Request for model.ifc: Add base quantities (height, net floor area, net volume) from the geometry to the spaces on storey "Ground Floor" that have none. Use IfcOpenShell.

First a look at what the model holds.

```python
import ifcopenshell
import ifcopenshell.util.element
import ifcopenshell.util.unit

model = ifcopenshell.open("model.ifc")
print(model.schema)
for unit_type in ("LENGTHUNIT", "AREAUNIT", "VOLUMEUNIT"):
    print(unit_type, ifcopenshell.util.unit.calculate_unit_scale(model, unit_type))
storey = next(s for s in model.by_type("IfcBuildingStorey") if s.Name == "Ground Floor")
spaces = [e for e in ifcopenshell.util.element.get_decomposition(storey) if e.is_a("IfcSpace")]
for e in sorted(spaces, key=lambda e: e.id()):
    print(e.id(), e.is_a(), e.Name, list(ifcopenshell.util.element.get_psets(e, qtos_only=True)), sep=" | ")
```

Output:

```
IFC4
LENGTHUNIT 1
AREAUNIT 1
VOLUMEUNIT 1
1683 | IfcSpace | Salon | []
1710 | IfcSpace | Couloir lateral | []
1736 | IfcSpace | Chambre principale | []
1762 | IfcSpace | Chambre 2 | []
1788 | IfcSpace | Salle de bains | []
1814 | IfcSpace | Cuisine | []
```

```python
import ifcopenshell
import ifcopenshell.api.pset
import ifcopenshell.geom
import ifcopenshell.util.element
import ifcopenshell.util.shape
import ifcopenshell.util.unit

model = ifcopenshell.open("model.ifc")
unit_scale = ifcopenshell.util.unit.calculate_unit_scale(model)
area_scale = ifcopenshell.util.unit.calculate_unit_scale(model, "AREAUNIT")
volume_scale = ifcopenshell.util.unit.calculate_unit_scale(model, "VOLUMEUNIT")
settings = ifcopenshell.geom.settings()

storey = next(s for s in model.by_type("IfcBuildingStorey") if s.Name == "Ground Floor")
spaces = [e for e in ifcopenshell.util.element.get_decomposition(storey) if e.is_a("IfcSpace")]

for e in sorted(spaces, key=lambda e: e.id()):
    if ifcopenshell.util.element.get_psets(e, qtos_only=True, should_inherit=False):
        continue
    # Geometry comes back in metres, in the element's own axes.
    shape = ifcopenshell.geom.create_shape(settings, e)
    values = {
        "Height": ifcopenshell.util.shape.get_z(shape.geometry) / unit_scale,
        "NetFloorArea": ifcopenshell.util.shape.get_footprint_area(shape.geometry) / area_scale,
        "NetVolume": ifcopenshell.util.shape.get_volume(shape.geometry) / volume_scale,
    }
    qto = ifcopenshell.api.pset.add_qto(model, product=e, name="Qto_SpaceBaseQuantities")
    ifcopenshell.api.pset.edit_qto(model, qto=qto, properties=values)
    print(e.id(), {k: round(v, 3) for k, v in values.items()})

model.write("model_v2.ifc")
```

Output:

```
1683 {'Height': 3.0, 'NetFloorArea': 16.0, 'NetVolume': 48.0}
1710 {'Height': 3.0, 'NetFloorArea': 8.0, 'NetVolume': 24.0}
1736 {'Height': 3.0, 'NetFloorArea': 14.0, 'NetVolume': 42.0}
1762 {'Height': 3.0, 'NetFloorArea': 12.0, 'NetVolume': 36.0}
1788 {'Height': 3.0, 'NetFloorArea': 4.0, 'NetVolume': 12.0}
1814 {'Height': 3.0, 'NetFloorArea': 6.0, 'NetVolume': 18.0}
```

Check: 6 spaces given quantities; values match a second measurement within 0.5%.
